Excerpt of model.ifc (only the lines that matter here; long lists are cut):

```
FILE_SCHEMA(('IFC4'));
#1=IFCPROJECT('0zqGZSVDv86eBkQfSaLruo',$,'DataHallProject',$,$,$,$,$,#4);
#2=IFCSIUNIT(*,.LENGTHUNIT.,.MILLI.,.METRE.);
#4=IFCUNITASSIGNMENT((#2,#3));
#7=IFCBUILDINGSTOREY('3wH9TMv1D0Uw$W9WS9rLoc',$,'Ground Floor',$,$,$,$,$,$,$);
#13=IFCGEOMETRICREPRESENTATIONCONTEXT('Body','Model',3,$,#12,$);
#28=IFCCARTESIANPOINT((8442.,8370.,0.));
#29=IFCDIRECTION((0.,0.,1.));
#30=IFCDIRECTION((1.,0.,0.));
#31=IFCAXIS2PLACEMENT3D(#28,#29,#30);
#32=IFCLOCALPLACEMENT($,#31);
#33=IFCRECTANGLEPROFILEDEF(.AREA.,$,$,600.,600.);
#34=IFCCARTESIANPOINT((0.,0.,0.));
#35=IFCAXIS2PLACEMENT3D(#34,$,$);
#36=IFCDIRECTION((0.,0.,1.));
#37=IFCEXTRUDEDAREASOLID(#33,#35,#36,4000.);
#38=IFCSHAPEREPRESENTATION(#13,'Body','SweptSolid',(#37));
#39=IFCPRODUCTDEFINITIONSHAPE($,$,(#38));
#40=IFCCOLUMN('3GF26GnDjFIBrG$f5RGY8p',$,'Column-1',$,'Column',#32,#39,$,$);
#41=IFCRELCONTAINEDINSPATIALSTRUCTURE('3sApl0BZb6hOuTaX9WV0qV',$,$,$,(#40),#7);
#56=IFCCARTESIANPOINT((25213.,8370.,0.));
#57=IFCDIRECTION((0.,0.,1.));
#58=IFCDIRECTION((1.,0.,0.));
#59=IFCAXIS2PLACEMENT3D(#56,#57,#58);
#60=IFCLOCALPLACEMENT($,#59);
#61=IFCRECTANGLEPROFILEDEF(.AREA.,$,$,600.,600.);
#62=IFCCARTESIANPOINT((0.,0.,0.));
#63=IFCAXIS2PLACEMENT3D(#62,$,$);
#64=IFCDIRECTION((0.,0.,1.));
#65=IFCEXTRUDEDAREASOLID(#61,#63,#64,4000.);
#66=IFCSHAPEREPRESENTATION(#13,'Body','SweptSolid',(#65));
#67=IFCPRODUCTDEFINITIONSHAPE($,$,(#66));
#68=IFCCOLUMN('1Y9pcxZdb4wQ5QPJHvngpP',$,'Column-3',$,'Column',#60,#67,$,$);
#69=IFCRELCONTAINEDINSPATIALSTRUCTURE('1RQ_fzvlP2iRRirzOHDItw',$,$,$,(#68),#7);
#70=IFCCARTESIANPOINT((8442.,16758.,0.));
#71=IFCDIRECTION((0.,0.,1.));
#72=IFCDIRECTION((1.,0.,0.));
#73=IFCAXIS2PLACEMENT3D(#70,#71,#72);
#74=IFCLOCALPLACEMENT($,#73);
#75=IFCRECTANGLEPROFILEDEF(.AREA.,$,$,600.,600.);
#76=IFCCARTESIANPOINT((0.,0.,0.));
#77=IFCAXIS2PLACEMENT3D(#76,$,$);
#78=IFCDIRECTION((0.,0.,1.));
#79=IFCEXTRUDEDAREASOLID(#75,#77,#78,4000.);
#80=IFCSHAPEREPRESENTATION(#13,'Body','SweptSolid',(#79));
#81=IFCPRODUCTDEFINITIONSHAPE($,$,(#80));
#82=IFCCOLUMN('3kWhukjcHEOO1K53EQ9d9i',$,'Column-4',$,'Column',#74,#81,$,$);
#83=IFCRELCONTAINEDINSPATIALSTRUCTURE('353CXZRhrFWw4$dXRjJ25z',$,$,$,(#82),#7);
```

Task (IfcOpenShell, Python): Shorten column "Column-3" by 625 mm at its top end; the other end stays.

```python
import ifcopenshell
import ifcopenshell.util.unit

model = ifcopenshell.open("model.ifc")
unit_scale = ifcopenshell.util.unit.calculate_unit_scale(model)

member = model.by_guid("1Y9pcxZdb4wQ5QPJHvngpP")
change = -0.625 / unit_scale

# The extrusion runs towards the end named, so only its depth changes.
body = next(r for r in member.Representation.Representations if r.RepresentationIdentifier == "Body")
solid = body.Items[0]
old_length = solid.Depth
solid.Depth += change

print(f"length {old_length:g} -> {solid.Depth:g}")

model.write("model_edited.ifc")
```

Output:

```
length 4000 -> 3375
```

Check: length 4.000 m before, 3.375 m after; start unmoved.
